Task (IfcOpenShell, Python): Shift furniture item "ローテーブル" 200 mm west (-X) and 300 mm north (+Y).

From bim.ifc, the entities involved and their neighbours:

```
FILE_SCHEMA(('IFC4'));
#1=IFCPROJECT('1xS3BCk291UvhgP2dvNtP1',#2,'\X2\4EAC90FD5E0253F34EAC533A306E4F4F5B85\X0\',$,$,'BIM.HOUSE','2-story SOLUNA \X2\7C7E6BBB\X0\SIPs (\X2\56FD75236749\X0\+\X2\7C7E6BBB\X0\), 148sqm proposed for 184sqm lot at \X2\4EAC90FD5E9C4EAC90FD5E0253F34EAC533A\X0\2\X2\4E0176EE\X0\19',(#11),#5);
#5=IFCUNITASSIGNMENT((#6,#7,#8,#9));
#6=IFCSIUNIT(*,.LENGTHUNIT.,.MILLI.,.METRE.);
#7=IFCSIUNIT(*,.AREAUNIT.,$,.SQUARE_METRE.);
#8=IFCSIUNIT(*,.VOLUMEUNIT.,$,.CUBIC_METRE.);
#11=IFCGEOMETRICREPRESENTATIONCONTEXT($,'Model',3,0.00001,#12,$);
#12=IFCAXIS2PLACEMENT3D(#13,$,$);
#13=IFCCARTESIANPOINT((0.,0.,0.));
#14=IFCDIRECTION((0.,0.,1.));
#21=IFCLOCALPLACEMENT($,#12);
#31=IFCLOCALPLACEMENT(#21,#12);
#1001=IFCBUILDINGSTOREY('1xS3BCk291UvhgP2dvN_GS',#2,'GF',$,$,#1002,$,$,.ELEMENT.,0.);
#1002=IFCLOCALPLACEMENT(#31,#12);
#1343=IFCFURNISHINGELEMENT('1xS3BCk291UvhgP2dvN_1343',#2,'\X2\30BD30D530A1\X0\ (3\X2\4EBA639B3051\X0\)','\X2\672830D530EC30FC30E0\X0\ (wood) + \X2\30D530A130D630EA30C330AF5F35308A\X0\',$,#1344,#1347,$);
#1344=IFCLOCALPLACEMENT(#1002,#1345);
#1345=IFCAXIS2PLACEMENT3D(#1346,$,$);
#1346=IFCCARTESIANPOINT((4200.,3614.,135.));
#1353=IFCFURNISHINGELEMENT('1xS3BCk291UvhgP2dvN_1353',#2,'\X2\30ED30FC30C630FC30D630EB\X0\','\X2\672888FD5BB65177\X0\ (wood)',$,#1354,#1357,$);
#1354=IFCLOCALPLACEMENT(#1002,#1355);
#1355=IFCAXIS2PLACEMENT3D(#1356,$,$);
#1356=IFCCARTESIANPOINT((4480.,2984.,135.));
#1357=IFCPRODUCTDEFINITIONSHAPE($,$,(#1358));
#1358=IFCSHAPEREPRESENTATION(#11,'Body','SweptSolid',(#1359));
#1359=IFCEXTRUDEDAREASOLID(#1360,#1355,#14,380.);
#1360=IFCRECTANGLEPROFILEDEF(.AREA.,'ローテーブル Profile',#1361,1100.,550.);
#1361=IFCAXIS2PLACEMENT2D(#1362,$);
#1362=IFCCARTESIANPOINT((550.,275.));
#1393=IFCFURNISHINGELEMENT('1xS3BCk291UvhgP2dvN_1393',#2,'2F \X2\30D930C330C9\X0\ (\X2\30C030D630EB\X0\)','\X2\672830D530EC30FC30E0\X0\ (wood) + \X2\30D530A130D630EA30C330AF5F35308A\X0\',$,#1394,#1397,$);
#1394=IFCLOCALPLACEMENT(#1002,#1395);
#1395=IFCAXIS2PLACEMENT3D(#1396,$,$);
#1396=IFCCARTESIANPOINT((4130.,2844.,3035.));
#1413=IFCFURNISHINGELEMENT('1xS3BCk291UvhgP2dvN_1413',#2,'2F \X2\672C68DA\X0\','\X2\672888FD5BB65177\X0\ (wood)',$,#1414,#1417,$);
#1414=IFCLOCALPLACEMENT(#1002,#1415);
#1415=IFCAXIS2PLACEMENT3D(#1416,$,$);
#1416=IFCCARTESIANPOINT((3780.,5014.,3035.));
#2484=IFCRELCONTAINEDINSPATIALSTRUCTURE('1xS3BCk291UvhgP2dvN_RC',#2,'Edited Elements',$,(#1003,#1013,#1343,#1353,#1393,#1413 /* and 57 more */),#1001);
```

```python
import ifcopenshell
import ifcopenshell.api.geometry
import ifcopenshell.util.placement

model = ifcopenshell.open("bim.ifc")

item = model.by_guid("1xS3BCk291UvhgP2dvN_1353")
matrix = ifcopenshell.util.placement.get_local_placement(item.ObjectPlacement)
matrix[0, 3] -= 200.0
matrix[1, 3] += 300.0
ifcopenshell.api.geometry.edit_object_placement(model, product=item, matrix=matrix, is_si=False)

print(ifcopenshell.util.placement.get_local_placement(item.ObjectPlacement).round(3) + 0.0)

model.write("bim_v2.ifc")
```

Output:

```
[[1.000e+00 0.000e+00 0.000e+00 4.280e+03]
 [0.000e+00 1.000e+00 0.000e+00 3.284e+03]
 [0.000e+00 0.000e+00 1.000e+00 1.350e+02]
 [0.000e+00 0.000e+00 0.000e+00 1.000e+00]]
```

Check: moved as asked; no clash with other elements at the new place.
